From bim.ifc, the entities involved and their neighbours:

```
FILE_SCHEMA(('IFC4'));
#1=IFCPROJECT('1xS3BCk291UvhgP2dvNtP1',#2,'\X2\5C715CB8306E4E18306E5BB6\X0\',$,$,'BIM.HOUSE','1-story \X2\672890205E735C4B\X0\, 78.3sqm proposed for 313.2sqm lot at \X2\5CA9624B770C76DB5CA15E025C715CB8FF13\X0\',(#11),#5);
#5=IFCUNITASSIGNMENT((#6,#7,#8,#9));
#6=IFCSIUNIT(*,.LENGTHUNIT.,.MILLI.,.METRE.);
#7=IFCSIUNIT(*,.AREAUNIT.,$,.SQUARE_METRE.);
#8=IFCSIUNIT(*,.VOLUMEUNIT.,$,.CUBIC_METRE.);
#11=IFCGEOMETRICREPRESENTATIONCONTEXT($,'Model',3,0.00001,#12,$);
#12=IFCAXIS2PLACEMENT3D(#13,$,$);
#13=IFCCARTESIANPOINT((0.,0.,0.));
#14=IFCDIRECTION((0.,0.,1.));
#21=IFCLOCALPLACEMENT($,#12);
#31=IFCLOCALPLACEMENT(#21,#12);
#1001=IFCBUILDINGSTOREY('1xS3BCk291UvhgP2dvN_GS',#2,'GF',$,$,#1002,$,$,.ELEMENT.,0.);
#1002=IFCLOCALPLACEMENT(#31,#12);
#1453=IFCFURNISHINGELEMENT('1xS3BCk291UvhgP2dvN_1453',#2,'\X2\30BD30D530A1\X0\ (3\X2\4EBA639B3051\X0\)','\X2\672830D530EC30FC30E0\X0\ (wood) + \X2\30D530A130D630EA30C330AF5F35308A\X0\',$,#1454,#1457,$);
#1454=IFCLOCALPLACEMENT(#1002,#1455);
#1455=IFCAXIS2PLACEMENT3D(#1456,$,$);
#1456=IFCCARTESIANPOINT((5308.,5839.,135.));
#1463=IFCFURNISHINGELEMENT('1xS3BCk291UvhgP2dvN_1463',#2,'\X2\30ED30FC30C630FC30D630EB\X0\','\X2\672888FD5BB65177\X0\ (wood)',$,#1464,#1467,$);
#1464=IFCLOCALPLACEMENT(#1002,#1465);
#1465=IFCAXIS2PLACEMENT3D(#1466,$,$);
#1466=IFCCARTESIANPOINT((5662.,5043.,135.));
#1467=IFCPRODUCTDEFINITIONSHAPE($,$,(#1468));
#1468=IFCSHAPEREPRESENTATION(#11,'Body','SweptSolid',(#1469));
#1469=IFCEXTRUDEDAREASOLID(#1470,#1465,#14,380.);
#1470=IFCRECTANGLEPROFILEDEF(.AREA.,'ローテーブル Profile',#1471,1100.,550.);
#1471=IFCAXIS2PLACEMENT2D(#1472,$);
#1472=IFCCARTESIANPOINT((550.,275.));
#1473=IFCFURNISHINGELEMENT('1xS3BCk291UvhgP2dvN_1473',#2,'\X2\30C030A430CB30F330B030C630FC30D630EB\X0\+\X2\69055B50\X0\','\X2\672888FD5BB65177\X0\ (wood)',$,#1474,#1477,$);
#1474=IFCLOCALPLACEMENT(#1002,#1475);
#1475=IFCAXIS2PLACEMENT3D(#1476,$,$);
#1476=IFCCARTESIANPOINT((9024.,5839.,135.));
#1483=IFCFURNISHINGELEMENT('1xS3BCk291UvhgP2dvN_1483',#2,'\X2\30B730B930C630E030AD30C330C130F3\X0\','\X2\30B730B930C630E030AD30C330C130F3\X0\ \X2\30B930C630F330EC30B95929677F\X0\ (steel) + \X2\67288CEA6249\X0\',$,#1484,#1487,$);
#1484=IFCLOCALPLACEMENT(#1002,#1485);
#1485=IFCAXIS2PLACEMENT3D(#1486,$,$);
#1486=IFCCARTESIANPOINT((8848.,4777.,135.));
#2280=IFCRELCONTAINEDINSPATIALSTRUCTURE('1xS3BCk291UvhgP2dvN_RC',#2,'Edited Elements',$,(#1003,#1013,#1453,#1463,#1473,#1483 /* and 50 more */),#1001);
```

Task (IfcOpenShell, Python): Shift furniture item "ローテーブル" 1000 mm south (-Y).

```python
import ifcopenshell
import ifcopenshell.api.geometry
import ifcopenshell.util.placement

model = ifcopenshell.open("bim.ifc")

item = model.by_guid("1xS3BCk291UvhgP2dvN_1463")
matrix = ifcopenshell.util.placement.get_local_placement(item.ObjectPlacement)
matrix[1, 3] -= 1000.0
ifcopenshell.api.geometry.edit_object_placement(model, product=item, matrix=matrix, is_si=False)

print(ifcopenshell.util.placement.get_local_placement(item.ObjectPlacement).round(3) + 0.0)

model.write("bim_rev.ifc")
```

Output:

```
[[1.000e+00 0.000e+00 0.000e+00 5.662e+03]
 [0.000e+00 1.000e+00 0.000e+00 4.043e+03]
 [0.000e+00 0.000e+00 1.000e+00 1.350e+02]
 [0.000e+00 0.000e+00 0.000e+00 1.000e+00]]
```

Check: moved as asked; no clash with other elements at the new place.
